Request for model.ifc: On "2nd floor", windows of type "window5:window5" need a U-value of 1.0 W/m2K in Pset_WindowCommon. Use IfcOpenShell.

First a look at what the model holds.

```python
import ifcopenshell
import ifcopenshell.util.element

model = ifcopenshell.open("model.ifc")
print(model.schema)
storey = next(s for s in model.by_type("IfcBuildingStorey") if s.Name == "2nd floor")
windows = [e for e in ifcopenshell.util.element.get_decomposition(storey) if e.is_a("IfcWindow")]
seen = {}
for e in windows:
    element_type = ifcopenshell.util.element.get_type(e)
    key = (element_type.Name if element_type != e and element_type else None, ifcopenshell.util.element.get_pset(e, "Pset_WindowCommon", "ThermalTransmittance"))
    seen[key] = seen.get(key, 0) + 1
for (name, value), count in sorted(seen.items(), key=str):
    print(count, "x", name, "|", value)
```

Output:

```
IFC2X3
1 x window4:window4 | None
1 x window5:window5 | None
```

```python
import ifcopenshell
import ifcopenshell.api.pset
import ifcopenshell.util.element

model = ifcopenshell.open("model.ifc")

storey = next(s for s in model.by_type("IfcBuildingStorey") if s.Name == "2nd floor")
windows = [e for e in ifcopenshell.util.element.get_decomposition(storey) if e.is_a("IfcWindow")]

count = 0
for e in windows:
    element_type = ifcopenshell.util.element.get_type(e)
    if element_type in (None, e) or element_type.Name != "window5:window5":
        continue
    # add_pset returns the element's existing set when there is one.
    pset = ifcopenshell.api.pset.add_pset(model, product=e, name="Pset_WindowCommon")
    ifcopenshell.api.pset.edit_pset(model, pset=pset, properties={"ThermalTransmittance": 1.0})
    count += 1

print(count, "windows updated")

model.write("model_v2.ifc")
```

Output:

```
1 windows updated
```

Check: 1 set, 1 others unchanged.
